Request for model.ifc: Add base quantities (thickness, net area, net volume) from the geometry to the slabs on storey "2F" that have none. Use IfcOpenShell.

First a look at what the model holds.

```python
import ifcopenshell
import ifcopenshell.util.element
import ifcopenshell.util.unit

model = ifcopenshell.open("model.ifc")
print(model.schema)
for unit_type in ("LENGTHUNIT", "AREAUNIT", "VOLUMEUNIT"):
    print(unit_type, ifcopenshell.util.unit.calculate_unit_scale(model, unit_type))
storey = next(s for s in model.by_type("IfcBuildingStorey") if s.Name == "2F")
slabs = [e for e in ifcopenshell.util.element.get_decomposition(storey) if e.is_a("IfcSlab")]
for e in sorted(slabs, key=lambda e: e.id()):
    print(e.id(), e.is_a(), e.Name, list(ifcopenshell.util.element.get_psets(e, qtos_only=True)), sep=" | ")
```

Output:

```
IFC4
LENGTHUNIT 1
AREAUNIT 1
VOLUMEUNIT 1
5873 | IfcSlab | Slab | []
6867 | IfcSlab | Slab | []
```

```python
import ifcopenshell
import ifcopenshell.api.pset
import ifcopenshell.geom
import ifcopenshell.util.element
import ifcopenshell.util.shape
import ifcopenshell.util.unit

model = ifcopenshell.open("model.ifc")
unit_scale = ifcopenshell.util.unit.calculate_unit_scale(model)
area_scale = ifcopenshell.util.unit.calculate_unit_scale(model, "AREAUNIT")
volume_scale = ifcopenshell.util.unit.calculate_unit_scale(model, "VOLUMEUNIT")
settings = ifcopenshell.geom.settings()

storey = next(s for s in model.by_type("IfcBuildingStorey") if s.Name == "2F")
slabs = [e for e in ifcopenshell.util.element.get_decomposition(storey) if e.is_a("IfcSlab")]

for e in sorted(slabs, key=lambda e: e.id()):
    if ifcopenshell.util.element.get_psets(e, qtos_only=True, should_inherit=False):
        continue
    # Geometry comes back in metres, in the element's own axes.
    shape = ifcopenshell.geom.create_shape(settings, e)
    values = {
        "Width": ifcopenshell.util.shape.get_z(shape.geometry) / unit_scale,
        "NetArea": ifcopenshell.util.shape.get_footprint_area(shape.geometry) / area_scale,
        "NetVolume": ifcopenshell.util.shape.get_volume(shape.geometry) / volume_scale,
    }
    qto = ifcopenshell.api.pset.add_qto(model, product=e, name="Qto_SlabBaseQuantities")
    ifcopenshell.api.pset.edit_qto(model, qto=qto, properties=values)
    print(e.id(), {k: round(v, 3) for k, v in values.items()})

model.write("model_updated.ifc")
```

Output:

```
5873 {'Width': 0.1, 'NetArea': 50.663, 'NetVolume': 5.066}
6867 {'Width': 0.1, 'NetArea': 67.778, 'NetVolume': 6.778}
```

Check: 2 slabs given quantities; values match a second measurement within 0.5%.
